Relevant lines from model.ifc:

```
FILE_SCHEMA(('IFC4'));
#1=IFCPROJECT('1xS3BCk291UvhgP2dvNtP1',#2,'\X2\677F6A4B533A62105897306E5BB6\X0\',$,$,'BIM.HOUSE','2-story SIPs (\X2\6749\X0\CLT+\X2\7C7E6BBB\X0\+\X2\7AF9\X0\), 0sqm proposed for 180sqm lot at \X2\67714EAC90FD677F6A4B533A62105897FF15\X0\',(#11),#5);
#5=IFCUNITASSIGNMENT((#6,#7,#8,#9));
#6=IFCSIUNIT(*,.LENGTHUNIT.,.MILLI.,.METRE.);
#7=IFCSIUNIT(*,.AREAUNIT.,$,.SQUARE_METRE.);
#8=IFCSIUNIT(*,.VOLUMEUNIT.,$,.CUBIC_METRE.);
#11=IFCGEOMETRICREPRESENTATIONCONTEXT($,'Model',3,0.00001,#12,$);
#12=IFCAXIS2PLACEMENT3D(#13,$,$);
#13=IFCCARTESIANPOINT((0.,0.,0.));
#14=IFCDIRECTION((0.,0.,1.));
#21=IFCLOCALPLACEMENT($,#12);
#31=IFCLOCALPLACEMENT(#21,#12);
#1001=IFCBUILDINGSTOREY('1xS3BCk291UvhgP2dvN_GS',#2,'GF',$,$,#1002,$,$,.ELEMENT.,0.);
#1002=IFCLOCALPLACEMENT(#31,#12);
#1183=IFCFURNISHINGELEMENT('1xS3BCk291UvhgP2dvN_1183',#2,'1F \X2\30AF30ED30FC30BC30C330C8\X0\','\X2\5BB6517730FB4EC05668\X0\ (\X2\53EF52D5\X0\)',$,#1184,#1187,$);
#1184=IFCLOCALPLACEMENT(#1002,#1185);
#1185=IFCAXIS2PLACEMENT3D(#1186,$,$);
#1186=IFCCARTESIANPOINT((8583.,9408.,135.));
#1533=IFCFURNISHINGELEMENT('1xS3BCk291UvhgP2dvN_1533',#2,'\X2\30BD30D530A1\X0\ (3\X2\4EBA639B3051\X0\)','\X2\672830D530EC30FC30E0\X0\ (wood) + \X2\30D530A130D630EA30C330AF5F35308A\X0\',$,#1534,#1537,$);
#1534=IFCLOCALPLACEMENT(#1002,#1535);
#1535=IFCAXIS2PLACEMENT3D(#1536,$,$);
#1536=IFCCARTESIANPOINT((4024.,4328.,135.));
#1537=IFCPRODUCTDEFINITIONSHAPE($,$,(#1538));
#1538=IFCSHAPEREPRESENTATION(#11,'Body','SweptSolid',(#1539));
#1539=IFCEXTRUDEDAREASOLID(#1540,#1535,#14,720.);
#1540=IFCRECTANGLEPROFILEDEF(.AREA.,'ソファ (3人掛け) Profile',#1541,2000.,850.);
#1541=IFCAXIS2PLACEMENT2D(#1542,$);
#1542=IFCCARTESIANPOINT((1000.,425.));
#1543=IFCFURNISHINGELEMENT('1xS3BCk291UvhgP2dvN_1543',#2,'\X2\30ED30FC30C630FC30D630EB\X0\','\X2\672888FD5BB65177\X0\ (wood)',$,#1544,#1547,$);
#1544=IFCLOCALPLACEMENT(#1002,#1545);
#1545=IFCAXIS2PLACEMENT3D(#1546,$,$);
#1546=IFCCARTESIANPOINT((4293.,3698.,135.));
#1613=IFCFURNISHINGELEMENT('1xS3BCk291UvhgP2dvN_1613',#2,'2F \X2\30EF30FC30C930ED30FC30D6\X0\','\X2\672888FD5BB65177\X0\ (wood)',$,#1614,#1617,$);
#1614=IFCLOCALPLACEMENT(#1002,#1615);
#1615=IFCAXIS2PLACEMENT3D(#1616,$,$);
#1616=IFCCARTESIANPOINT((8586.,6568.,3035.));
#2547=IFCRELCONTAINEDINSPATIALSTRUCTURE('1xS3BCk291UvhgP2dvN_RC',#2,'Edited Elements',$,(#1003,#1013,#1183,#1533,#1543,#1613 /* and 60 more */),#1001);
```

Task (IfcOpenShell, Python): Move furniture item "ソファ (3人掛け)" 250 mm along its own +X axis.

```python
import ifcopenshell
import ifcopenshell.api.geometry
import ifcopenshell.util.placement
import ifcopenshell.util.unit

model = ifcopenshell.open("model.ifc")
unit_scale = ifcopenshell.util.unit.calculate_unit_scale(model)

item = model.by_guid("1xS3BCk291UvhgP2dvN_1533")
matrix = ifcopenshell.util.placement.get_local_placement(item.ObjectPlacement)
matrix[:3, 3] += matrix[:3, 0] * 0.25 / unit_scale
ifcopenshell.api.geometry.edit_object_placement(model, product=item, matrix=matrix, is_si=False)

print(ifcopenshell.util.placement.get_local_placement(item.ObjectPlacement).round(3) + 0.0)

model.write("model_rev.ifc")
```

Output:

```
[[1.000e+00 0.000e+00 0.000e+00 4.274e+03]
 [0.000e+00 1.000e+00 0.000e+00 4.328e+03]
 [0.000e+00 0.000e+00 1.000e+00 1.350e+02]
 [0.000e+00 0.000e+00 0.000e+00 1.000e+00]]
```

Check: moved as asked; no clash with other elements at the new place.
